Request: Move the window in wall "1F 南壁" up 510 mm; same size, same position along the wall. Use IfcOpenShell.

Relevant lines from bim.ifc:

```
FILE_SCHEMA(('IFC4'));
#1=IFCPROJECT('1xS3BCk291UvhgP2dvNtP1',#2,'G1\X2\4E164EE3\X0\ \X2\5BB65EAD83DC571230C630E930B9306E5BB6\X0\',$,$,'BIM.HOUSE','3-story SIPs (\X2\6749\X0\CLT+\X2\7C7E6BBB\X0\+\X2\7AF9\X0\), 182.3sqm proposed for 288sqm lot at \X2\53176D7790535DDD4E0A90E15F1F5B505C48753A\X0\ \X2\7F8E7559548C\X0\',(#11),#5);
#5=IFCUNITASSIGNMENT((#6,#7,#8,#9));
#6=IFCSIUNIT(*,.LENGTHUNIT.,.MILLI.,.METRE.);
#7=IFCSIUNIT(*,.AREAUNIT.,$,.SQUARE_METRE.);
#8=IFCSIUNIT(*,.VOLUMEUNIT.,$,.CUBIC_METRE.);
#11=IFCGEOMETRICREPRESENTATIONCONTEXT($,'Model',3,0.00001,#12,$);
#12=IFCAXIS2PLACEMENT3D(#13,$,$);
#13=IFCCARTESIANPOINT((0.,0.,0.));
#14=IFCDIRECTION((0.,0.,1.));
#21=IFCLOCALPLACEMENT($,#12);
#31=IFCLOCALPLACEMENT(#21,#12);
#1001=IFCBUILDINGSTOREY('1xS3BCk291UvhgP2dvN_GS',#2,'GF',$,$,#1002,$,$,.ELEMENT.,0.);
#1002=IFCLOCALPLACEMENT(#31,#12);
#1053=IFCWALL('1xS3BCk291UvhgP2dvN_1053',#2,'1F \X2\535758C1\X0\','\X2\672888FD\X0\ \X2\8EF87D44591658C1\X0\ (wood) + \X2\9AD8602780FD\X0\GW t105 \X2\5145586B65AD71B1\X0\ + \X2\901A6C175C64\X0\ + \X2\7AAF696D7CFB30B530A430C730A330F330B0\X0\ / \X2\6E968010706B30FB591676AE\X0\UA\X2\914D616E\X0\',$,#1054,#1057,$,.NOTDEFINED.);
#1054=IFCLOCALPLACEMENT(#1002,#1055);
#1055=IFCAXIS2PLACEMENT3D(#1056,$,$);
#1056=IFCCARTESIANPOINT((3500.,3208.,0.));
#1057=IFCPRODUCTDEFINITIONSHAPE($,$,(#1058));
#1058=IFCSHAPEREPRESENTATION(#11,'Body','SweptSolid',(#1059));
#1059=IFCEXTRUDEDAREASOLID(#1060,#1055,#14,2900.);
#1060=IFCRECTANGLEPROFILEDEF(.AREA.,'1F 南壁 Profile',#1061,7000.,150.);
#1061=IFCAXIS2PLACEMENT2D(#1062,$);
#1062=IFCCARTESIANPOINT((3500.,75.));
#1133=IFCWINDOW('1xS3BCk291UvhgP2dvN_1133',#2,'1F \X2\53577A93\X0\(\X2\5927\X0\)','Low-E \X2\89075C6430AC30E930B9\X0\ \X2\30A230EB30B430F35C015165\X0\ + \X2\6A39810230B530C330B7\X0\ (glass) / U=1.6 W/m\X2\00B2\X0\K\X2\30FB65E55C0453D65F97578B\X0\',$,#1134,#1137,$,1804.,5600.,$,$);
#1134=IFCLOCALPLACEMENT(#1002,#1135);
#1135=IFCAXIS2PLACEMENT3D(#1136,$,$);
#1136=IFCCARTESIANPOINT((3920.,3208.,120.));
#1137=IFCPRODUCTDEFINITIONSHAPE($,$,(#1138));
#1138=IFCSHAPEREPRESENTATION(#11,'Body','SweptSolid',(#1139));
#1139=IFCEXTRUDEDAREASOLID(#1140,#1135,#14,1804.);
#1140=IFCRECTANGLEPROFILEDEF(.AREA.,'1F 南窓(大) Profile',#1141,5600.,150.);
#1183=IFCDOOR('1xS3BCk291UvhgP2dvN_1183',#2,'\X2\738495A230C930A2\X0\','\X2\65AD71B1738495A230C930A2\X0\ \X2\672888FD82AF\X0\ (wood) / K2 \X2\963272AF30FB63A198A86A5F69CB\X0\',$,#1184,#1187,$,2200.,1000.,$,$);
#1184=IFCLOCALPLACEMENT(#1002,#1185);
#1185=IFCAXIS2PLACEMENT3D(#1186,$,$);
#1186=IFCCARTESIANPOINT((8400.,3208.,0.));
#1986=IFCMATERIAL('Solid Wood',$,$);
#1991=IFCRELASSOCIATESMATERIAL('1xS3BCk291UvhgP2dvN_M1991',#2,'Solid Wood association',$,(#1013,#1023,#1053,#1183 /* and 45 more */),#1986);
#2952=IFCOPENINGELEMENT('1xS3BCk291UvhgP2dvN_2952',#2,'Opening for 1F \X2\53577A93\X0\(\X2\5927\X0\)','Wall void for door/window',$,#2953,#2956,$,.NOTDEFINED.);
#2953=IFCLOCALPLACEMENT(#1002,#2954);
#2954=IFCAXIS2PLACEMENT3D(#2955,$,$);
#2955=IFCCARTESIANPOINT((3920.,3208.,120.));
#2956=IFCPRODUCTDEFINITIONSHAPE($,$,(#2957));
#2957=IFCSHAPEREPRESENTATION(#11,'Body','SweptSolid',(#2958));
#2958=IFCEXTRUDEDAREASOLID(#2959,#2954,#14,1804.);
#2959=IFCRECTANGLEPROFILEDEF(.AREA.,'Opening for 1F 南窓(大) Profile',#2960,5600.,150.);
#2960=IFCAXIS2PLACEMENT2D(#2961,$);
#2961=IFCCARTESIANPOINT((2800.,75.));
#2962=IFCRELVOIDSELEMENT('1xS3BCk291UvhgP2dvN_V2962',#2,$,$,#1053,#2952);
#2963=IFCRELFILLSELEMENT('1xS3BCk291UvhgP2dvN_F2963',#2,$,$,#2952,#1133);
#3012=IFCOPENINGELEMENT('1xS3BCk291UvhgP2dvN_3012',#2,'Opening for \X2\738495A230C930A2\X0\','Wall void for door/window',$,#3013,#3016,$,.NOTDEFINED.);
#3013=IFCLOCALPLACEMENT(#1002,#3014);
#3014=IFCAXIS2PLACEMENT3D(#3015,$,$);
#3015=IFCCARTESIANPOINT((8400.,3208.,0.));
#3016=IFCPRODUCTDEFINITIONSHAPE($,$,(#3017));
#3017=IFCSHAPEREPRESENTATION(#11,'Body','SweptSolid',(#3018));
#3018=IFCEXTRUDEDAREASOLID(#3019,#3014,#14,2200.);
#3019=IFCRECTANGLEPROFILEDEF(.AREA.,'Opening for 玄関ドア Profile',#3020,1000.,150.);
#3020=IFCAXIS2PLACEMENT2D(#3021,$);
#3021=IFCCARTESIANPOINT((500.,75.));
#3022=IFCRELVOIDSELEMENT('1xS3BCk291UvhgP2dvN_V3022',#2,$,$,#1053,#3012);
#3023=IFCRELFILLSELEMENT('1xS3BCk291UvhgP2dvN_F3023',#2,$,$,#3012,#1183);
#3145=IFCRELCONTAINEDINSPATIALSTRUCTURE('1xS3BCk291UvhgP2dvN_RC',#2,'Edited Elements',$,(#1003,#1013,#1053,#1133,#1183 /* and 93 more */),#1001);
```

```python
import numpy as np
import ifcopenshell
import ifcopenshell.api.geometry
import ifcopenshell.util.placement
import ifcopenshell.util.unit

model = ifcopenshell.open("bim.ifc")
unit_scale = ifcopenshell.util.unit.calculate_unit_scale(model)

window = model.by_guid("1xS3BCk291UvhgP2dvN_1133")
opening = window.FillsVoids[0].RelatingOpeningElement
dz = 510.0

shift = np.array([0.0, 0.0, dz])
# The window is not placed relative to its opening, so move both.
for product in (opening, window):
    matrix = ifcopenshell.util.placement.get_local_placement(product.ObjectPlacement)
    matrix[:3, 3] += shift
    ifcopenshell.api.geometry.edit_object_placement(model, product=product, matrix=matrix, is_si=False)

print(f"moved by {dz * unit_scale:+.3f} m")

model.write("bim-out.ifc")
```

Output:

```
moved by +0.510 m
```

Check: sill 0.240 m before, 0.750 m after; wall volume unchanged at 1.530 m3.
